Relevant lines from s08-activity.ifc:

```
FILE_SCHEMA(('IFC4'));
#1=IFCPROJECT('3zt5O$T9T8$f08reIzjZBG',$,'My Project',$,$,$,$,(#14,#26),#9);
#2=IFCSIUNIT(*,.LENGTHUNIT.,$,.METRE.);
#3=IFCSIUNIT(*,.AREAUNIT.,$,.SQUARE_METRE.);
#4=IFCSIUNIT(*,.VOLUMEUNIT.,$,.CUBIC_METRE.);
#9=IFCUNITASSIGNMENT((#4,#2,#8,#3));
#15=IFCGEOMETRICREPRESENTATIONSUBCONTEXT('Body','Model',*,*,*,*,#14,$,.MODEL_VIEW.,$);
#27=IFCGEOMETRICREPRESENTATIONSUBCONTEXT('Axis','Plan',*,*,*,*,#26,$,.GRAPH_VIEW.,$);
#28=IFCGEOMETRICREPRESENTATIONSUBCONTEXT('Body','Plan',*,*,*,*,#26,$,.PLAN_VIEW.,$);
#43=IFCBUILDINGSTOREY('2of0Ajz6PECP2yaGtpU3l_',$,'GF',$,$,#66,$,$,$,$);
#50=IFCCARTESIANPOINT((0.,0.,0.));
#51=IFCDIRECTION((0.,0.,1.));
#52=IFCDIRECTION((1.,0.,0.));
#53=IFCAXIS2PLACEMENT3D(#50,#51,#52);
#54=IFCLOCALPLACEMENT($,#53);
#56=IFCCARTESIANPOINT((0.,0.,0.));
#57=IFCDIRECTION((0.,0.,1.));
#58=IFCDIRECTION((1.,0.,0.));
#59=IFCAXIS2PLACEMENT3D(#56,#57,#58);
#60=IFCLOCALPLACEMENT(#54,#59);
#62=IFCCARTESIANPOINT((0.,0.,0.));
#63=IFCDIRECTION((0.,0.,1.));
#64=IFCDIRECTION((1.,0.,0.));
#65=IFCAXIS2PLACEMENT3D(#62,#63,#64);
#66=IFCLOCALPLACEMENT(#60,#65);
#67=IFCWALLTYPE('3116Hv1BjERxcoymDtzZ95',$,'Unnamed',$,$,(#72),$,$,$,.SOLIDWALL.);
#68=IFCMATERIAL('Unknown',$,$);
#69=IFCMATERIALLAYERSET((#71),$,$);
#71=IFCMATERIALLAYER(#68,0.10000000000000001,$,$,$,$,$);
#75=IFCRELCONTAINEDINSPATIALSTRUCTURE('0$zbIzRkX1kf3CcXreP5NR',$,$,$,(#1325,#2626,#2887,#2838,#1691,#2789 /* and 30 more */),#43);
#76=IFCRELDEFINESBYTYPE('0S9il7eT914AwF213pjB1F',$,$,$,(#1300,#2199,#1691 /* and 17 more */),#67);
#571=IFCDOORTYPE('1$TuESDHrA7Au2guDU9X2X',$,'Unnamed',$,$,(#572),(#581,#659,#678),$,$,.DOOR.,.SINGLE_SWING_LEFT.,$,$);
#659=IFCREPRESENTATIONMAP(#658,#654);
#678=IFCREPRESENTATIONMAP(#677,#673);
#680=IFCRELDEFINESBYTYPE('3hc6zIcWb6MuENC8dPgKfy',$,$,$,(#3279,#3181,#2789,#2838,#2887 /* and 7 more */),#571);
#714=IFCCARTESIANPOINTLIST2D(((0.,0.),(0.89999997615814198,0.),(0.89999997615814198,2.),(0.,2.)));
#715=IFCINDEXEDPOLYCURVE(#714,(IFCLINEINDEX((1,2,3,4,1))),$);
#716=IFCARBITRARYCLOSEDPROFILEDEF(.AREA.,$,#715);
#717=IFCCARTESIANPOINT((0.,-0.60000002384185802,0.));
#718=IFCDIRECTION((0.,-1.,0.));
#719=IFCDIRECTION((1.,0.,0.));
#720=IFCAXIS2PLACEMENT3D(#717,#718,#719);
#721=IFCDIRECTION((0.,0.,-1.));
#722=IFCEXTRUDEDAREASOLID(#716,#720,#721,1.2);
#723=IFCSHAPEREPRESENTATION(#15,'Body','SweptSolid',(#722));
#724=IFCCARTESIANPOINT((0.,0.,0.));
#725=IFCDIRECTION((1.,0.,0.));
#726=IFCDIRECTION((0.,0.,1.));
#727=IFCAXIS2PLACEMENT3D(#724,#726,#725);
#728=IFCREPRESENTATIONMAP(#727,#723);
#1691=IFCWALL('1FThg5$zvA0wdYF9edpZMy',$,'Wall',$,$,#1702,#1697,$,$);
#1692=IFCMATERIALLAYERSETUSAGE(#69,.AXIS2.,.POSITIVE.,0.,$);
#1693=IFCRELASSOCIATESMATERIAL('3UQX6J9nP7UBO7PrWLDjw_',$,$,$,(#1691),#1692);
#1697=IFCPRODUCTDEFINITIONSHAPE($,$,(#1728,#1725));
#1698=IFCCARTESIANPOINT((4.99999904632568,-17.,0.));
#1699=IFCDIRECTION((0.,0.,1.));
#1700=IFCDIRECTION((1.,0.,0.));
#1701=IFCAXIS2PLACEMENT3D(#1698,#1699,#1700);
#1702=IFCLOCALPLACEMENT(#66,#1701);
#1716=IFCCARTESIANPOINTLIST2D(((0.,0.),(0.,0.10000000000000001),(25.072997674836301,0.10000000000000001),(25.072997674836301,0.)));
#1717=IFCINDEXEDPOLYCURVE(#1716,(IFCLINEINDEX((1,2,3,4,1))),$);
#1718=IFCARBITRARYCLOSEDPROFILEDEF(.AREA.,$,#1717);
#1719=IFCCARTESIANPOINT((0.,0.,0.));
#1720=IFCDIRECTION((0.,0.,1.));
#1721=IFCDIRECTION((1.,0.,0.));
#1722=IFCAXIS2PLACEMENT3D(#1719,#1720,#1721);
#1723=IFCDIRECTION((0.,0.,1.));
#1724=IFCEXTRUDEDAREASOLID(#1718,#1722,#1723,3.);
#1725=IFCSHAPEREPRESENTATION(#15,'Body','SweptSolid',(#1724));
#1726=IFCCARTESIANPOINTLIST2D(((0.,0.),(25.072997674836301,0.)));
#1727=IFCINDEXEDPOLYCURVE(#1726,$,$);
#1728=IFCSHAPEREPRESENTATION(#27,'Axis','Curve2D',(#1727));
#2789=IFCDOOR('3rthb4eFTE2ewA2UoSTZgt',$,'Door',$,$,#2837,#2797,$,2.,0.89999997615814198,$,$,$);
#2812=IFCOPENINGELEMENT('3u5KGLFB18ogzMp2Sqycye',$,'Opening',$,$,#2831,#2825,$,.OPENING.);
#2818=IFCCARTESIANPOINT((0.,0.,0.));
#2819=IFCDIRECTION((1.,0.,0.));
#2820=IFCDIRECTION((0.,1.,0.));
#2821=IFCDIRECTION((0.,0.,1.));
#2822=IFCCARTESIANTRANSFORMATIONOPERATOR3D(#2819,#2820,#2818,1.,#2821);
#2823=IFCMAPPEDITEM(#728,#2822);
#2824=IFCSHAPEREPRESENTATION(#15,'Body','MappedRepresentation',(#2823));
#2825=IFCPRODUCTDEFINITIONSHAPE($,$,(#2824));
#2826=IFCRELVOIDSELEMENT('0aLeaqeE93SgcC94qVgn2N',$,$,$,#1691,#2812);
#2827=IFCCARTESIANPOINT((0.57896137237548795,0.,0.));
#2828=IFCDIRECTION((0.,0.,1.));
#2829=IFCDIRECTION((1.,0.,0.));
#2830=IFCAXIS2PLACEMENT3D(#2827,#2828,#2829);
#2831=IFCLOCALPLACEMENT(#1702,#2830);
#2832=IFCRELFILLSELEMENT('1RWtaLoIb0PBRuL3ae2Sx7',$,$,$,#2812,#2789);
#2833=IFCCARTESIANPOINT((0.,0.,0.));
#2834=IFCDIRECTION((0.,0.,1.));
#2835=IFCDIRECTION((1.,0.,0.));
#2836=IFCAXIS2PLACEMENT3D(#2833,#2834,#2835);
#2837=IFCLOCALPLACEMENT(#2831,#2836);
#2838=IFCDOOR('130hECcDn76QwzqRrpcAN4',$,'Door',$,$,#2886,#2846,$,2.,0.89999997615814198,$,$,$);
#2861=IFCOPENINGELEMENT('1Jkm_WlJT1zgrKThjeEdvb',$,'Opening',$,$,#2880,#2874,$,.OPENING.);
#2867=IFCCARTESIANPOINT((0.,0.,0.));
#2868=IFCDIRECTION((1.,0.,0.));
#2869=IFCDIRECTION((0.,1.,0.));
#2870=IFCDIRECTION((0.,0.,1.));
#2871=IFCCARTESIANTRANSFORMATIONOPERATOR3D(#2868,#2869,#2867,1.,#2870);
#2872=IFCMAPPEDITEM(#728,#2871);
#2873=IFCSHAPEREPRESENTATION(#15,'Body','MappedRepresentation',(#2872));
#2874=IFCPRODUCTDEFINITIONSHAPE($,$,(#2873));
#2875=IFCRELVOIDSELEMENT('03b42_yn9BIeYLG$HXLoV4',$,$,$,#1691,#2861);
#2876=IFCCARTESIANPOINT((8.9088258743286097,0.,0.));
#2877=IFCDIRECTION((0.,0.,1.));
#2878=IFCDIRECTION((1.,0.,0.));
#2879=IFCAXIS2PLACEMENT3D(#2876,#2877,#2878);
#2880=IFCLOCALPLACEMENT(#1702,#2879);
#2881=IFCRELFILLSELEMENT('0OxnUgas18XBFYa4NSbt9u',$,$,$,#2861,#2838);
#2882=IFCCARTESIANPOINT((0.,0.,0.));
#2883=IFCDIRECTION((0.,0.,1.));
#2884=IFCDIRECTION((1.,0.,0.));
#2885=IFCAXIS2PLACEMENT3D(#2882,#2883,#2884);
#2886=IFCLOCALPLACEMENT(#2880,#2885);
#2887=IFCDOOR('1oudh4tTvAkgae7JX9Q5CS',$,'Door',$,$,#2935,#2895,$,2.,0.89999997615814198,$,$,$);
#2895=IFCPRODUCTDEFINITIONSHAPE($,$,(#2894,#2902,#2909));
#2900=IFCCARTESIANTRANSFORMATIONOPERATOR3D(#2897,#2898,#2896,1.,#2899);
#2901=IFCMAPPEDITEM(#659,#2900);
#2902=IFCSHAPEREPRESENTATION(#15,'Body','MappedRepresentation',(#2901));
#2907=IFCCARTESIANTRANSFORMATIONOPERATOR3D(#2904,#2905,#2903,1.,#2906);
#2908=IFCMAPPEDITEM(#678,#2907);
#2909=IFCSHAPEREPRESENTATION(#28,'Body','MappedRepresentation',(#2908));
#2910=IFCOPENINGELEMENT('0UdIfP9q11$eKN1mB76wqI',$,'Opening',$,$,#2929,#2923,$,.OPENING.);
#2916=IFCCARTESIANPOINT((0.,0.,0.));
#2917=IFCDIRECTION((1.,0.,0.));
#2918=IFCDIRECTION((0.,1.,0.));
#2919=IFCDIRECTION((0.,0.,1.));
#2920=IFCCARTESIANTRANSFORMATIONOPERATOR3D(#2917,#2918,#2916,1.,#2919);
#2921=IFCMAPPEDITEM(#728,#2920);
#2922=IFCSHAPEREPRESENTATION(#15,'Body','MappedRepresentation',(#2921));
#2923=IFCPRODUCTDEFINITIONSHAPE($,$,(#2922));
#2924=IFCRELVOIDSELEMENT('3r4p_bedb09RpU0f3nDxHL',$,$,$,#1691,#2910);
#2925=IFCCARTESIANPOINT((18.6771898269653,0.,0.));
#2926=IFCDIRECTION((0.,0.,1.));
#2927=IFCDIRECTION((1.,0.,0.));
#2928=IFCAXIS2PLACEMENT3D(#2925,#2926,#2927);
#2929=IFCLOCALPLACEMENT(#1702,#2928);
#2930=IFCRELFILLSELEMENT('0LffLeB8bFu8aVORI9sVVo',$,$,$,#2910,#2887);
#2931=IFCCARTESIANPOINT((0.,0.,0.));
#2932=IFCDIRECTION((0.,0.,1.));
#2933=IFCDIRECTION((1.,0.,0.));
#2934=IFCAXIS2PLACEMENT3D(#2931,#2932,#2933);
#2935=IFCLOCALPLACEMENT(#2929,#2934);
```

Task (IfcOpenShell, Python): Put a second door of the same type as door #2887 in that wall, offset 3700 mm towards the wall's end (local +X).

```python
import ifcopenshell
import ifcopenshell.api.feature
import ifcopenshell.api.geometry
import ifcopenshell.api.root
import ifcopenshell.geom
import ifcopenshell.util.element
import ifcopenshell.util.placement
import ifcopenshell.util.shape
import ifcopenshell.util.unit

model = ifcopenshell.open("s08-activity.ifc")
unit_scale = ifcopenshell.util.unit.calculate_unit_scale(model)
settings = ifcopenshell.geom.settings()


def volume(element):
    """Net volume in cubic metres, openings subtracted."""
    shape = ifcopenshell.geom.create_shape(settings, element)
    return ifcopenshell.util.shape.get_volume(shape.geometry)


door = model.by_id(2887)
opening = door.FillsVoids[0].RelatingOpeningElement
wall = opening.VoidsElements[0].RelatingBuildingElement
before = volume(wall)
shift = ifcopenshell.util.placement.get_local_placement(wall.ObjectPlacement)[:3, 0] * 3.7 / unit_scale

# copy_class copies the void relationship, type, container and properties, but no geometry.
new_opening = ifcopenshell.api.root.copy_class(model, product=opening)
new_opening.Representation = ifcopenshell.util.element.copy_deep(
    model, opening.Representation, exclude=["IfcGeometricRepresentationContext", "IfcRepresentationMap"]
)
new_door = ifcopenshell.api.root.copy_class(model, product=door)
new_door.Representation = ifcopenshell.util.element.copy_deep(
    model, door.Representation, exclude=["IfcGeometricRepresentationContext", "IfcRepresentationMap"]
)
ifcopenshell.api.feature.add_filling(model, opening=new_opening, element=new_door)

for old, new in ((opening, new_opening), (door, new_door)):
    matrix = ifcopenshell.util.placement.get_local_placement(old.ObjectPlacement)
    matrix[:3, 3] += shift
    ifcopenshell.api.geometry.edit_object_placement(model, product=new, matrix=matrix, is_si=False)

after = volume(wall)

print(f"wall volume {before:.3f} -> {after:.3f} m3")

model.write("s08-activity-out.ifc")
```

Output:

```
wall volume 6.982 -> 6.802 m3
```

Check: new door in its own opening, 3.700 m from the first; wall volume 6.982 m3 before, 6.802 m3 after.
